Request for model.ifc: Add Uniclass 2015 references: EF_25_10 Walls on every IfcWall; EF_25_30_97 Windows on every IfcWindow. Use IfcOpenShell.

First a look at what the model holds.

```python
import ifcopenshell

model = ifcopenshell.open("model.ifc")
print(model.schema)
print("classifications:", [c.Name for c in model.by_type("IfcClassification")])
for ifc_class in ("IfcDoor", "IfcRoof", "IfcStair", "IfcWall", "IfcWindow"):
    print(ifc_class, len(model.by_type(ifc_class)))
```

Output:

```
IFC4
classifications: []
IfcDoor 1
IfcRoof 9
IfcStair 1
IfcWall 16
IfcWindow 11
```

```python
import ifcopenshell
import ifcopenshell.api.classification

model = ifcopenshell.open("model.ifc")

system = ifcopenshell.api.classification.add_classification(model, classification="Uniclass 2015")

codes = {
    "IfcWall": ("EF_25_10", "Walls"),
    "IfcWindow": ("EF_25_30_97", "Windows"),
}
for ifc_class, (code, name) in codes.items():
    products = model.by_type(ifc_class)
    ifcopenshell.api.classification.add_reference(
        model, products=products, classification=system, identification=code, name=name
    )
    print(code, len(products))

model.write("model_v2.ifc")
```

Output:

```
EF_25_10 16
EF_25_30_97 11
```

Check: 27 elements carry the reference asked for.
